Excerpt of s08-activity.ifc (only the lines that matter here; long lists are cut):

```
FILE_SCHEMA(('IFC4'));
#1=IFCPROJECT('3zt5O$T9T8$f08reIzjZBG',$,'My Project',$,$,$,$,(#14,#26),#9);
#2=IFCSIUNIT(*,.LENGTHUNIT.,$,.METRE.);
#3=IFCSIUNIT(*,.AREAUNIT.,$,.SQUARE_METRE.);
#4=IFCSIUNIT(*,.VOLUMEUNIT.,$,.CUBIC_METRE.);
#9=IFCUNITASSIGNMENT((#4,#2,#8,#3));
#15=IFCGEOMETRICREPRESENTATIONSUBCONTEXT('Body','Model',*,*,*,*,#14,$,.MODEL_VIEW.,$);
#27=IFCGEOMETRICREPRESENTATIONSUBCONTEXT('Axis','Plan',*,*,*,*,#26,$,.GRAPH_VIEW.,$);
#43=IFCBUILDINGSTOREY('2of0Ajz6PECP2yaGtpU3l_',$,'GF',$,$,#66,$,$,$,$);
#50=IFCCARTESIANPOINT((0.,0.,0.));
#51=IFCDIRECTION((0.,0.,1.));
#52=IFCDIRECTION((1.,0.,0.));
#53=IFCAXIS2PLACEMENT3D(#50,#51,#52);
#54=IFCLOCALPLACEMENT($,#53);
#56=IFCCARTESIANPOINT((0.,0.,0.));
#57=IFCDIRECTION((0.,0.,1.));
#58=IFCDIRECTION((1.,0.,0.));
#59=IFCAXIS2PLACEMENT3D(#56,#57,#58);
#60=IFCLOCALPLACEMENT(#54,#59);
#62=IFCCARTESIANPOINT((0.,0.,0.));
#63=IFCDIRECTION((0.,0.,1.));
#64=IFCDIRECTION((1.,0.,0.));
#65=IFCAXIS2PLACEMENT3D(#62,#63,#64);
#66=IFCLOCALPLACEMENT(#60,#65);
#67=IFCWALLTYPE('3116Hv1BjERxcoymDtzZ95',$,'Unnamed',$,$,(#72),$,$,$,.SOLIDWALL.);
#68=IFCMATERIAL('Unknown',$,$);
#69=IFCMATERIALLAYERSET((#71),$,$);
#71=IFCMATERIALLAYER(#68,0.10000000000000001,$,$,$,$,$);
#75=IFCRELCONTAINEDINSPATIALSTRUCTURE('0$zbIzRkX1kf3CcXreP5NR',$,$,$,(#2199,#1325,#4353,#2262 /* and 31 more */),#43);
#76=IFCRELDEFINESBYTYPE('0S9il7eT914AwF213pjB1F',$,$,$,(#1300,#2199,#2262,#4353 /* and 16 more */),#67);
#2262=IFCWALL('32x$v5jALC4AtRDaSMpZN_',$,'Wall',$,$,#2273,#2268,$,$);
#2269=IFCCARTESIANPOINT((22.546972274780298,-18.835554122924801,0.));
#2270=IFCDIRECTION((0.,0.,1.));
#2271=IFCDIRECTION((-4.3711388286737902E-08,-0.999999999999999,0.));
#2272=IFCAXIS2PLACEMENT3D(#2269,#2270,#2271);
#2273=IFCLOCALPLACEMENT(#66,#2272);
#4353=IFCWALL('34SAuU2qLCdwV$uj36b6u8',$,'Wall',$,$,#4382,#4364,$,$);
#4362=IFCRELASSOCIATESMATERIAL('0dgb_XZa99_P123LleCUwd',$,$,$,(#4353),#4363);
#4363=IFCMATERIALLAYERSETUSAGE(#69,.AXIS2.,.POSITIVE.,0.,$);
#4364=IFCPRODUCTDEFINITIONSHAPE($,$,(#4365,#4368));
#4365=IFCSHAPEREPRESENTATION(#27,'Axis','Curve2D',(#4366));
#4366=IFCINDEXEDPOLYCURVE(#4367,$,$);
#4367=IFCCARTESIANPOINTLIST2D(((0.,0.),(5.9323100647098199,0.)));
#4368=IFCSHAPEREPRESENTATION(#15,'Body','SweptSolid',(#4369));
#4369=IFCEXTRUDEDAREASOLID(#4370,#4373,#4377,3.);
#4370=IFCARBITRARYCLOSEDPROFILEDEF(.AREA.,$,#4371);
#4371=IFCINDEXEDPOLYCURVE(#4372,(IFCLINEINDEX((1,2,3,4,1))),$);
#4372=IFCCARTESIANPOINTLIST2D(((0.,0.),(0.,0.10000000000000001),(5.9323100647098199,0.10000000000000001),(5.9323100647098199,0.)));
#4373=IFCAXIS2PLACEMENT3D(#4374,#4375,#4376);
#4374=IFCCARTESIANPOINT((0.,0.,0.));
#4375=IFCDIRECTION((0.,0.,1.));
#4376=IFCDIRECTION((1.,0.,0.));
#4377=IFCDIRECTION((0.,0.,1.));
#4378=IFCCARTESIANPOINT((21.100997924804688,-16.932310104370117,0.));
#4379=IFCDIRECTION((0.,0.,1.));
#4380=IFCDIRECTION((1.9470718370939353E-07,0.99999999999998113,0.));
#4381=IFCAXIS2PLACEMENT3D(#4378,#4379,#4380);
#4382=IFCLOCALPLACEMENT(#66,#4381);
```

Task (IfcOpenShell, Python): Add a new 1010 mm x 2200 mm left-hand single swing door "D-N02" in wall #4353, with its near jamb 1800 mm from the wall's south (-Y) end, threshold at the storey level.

```python
import numpy as np
import ifcopenshell
import ifcopenshell.api.feature
import ifcopenshell.api.geometry
import ifcopenshell.api.root
import ifcopenshell.api.spatial
import ifcopenshell.geom
import ifcopenshell.util.element
import ifcopenshell.util.placement
import ifcopenshell.util.representation
import ifcopenshell.util.shape
import ifcopenshell.util.unit

model = ifcopenshell.open("s08-activity.ifc")
unit_scale = ifcopenshell.util.unit.calculate_unit_scale(model)
settings = ifcopenshell.geom.settings()


def volume(element):
    """Net volume in cubic metres, openings subtracted."""
    shape = ifcopenshell.geom.create_shape(settings, element)
    return ifcopenshell.util.shape.get_volume(shape.geometry)


wall = model.by_guid("34SAuU2qLCdwV$uj36b6u8")
storey = ifcopenshell.util.element.get_container(wall, ifc_class="IfcBuildingStorey")
context = ifcopenshell.util.representation.get_context(model, "Model", "Body", "MODEL_VIEW")
before = volume(wall)

width, height, from_end, sill = 1.01, 2.2, 1.8, 0.0  # metres

# The wall runs along its own X axis, and the end named is its -X end.
wall_shape = ifcopenshell.geom.create_shape(settings, wall)
x, y, z = ifcopenshell.util.shape.get_vertices(wall_shape.geometry).T
start = x.min() + from_end
face, thickness = float(y.min()), float(y.max() - y.min())
wall_matrix = ifcopenshell.util.placement.get_local_placement(wall.ObjectPlacement)
level = ifcopenshell.util.placement.get_local_placement(storey.ObjectPlacement)[2, 3]


def in_wall(x, y):
    """Placement at x, y metres in the wall's axes, at sill height."""
    matrix = wall_matrix.copy()
    matrix[:, 3] = wall_matrix @ np.array([x / unit_scale, y / unit_scale, 0.0, 1.0])
    matrix[2, 3] = level + sill / unit_scale
    return matrix


# Opening: a box that overshoots both wall faces by 50 mm.
opening = ifcopenshell.api.root.create_entity(model, ifc_class="IfcOpeningElement", predefined_type="OPENING")
box = ifcopenshell.api.geometry.add_wall_representation(
    model, context=context, length=width, height=height, thickness=thickness + 0.1
)
ifcopenshell.api.geometry.assign_representation(model, product=opening, representation=box)
ifcopenshell.api.geometry.edit_object_placement(model, product=opening, matrix=in_wall(start, face - 0.05), is_si=False)
ifcopenshell.api.feature.add_feature(model, feature=opening, element=wall)

door = ifcopenshell.api.root.create_entity(model, ifc_class="IfcDoor", name="D-N02", predefined_type="DOOR")
door.OverallWidth, door.OverallHeight = width / unit_scale, height / unit_scale
door.OperationType = "SINGLE_SWING_LEFT"
body = ifcopenshell.api.geometry.add_door_representation(
    model,
    context=context,
    overall_width=door.OverallWidth,
    overall_height=door.OverallHeight,
    operation_type="SINGLE_SWING_LEFT",
    lining_properties={"LiningDepth": thickness / unit_scale, "ThresholdDepth": thickness / unit_scale},
)
ifcopenshell.api.geometry.assign_representation(model, product=door, representation=body)
ifcopenshell.api.spatial.assign_container(model, products=[door], relating_structure=storey)
ifcopenshell.api.feature.add_filling(model, opening=opening, element=door)

# The lining spans the wall, so the door starts at the wall face.
ifcopenshell.api.geometry.edit_object_placement(model, product=door, matrix=in_wall(start, face), is_si=False)

after = volume(wall)

print(f"wall volume {before:.3f} -> {after:.3f} m3")

model.write("s08-activity-out.ifc")
```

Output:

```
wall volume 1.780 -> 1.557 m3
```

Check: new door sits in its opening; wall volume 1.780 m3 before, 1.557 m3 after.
